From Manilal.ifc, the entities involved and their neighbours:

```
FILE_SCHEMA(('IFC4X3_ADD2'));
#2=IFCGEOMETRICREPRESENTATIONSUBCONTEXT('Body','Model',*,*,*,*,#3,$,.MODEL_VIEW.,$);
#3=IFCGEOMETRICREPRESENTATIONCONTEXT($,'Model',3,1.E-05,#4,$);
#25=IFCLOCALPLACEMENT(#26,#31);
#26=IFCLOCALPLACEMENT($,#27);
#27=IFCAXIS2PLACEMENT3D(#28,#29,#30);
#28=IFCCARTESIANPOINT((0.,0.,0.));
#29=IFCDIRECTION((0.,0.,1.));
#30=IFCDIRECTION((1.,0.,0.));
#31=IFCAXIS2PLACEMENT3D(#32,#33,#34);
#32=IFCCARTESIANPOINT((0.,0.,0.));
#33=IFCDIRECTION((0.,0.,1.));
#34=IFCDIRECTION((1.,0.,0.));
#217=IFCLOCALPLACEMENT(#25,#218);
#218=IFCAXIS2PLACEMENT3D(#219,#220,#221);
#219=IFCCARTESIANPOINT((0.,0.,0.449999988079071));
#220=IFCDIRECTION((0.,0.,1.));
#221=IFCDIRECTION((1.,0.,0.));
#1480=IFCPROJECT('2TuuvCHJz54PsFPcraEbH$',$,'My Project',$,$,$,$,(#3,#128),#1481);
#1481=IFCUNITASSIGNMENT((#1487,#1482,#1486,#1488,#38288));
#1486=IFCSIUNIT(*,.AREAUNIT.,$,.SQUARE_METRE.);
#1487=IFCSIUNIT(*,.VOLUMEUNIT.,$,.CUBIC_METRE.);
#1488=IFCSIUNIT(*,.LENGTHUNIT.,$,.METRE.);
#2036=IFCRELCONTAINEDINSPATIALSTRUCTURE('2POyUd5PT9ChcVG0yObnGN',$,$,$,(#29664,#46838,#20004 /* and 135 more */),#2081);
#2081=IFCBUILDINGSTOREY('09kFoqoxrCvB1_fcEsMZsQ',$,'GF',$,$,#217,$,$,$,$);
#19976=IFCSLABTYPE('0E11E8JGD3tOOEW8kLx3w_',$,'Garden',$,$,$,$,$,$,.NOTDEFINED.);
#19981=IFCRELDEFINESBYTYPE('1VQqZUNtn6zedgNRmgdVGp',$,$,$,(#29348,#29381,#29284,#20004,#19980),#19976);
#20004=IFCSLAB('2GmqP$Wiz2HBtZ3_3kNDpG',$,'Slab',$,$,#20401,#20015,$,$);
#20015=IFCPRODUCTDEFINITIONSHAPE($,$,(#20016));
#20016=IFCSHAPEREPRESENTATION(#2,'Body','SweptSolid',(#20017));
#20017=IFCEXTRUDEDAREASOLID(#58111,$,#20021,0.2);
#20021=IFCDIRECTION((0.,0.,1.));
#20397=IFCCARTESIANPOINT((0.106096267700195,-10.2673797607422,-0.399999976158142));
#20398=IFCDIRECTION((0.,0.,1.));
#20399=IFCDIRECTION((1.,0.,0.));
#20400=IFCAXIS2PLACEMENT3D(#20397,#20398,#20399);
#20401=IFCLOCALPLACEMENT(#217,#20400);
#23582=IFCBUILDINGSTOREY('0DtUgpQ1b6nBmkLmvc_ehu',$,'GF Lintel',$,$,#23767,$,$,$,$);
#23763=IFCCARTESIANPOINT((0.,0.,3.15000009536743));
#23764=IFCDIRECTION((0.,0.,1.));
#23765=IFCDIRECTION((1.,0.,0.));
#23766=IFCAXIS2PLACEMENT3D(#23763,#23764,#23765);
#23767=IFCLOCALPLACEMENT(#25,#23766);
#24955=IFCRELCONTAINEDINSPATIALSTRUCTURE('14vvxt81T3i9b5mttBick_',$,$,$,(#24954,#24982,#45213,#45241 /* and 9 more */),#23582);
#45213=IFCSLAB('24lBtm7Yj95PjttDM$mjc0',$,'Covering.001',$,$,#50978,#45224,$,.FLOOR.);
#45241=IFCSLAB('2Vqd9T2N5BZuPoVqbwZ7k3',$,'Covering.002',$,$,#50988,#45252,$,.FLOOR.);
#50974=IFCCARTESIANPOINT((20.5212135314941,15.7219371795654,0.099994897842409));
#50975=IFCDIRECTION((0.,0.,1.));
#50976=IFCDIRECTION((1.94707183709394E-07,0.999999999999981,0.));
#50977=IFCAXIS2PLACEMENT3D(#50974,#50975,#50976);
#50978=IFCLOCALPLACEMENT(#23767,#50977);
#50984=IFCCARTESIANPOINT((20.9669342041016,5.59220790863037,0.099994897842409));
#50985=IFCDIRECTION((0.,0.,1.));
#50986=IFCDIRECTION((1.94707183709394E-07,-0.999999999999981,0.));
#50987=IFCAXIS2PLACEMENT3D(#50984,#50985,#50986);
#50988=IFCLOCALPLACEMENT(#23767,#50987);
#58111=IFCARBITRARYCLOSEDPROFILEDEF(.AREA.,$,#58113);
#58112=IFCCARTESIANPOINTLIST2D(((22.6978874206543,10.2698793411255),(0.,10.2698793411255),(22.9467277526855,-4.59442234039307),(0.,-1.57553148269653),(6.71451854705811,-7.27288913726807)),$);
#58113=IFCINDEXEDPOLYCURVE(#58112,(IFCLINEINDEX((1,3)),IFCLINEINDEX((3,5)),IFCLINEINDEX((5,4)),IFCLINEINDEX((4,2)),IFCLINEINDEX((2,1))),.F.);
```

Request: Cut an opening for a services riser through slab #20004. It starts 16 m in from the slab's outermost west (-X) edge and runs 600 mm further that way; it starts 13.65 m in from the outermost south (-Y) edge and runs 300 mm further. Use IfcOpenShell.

```python
import numpy as np
import ifcopenshell
import ifcopenshell.api.feature
import ifcopenshell.api.geometry
import ifcopenshell.api.root
import ifcopenshell.geom
import ifcopenshell.util.placement
import ifcopenshell.util.representation
import ifcopenshell.util.shape
import ifcopenshell.util.unit

model = ifcopenshell.open("Manilal.ifc")
unit_scale = ifcopenshell.util.unit.calculate_unit_scale(model)
settings = ifcopenshell.geom.settings()


def volume(element):
    """Net volume in cubic metres, openings subtracted."""
    shape = ifcopenshell.geom.create_shape(settings, element)
    return ifcopenshell.util.shape.get_volume(shape.geometry)


slab = model.by_id(20004)
before = volume(slab)

# Extent in the slab's own axes, in metres. The edges named are its -X and -Y sides.
slab_shape = ifcopenshell.geom.create_shape(settings, slab)
vertices = ifcopenshell.util.shape.get_vertices(slab_shape.geometry)
x_min, y_min, bottom = vertices.min(axis=0)
top = vertices[:, 2].max()

opening = ifcopenshell.api.root.create_entity(model, ifc_class="IfcOpeningElement", name="Services riser opening", predefined_type="OPENING")
context = ifcopenshell.util.representation.get_context(model, "Model", "Body", "MODEL_VIEW")
width, depth = 0.6, 0.3
outline = [(0.0, 0.0), (width, 0.0), (width, depth), (0.0, depth), (0.0, 0.0)]
# Overshoot both faces by 50 mm so the cut is clean.
shape = ifcopenshell.api.geometry.add_slab_representation(
    model, context=context, depth=top - bottom + 0.1, polyline=outline
)
ifcopenshell.api.geometry.assign_representation(model, product=opening, representation=shape)

matrix = ifcopenshell.util.placement.get_local_placement(slab.ObjectPlacement)
matrix[:, 3] = matrix @ np.append(np.array([x_min + 16, y_min + 13.65, bottom - 0.05]) / unit_scale, 1.0)
ifcopenshell.api.geometry.edit_object_placement(model, product=opening, matrix=matrix, is_si=False)
ifcopenshell.api.feature.add_feature(model, feature=opening, element=slab)

after = volume(slab)

print(f"slab volume {before:.3f} -> {after:.3f} m3")

model.write("Manilal_v2.ifc")
```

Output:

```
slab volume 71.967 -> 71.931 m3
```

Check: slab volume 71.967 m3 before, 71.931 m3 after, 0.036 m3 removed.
